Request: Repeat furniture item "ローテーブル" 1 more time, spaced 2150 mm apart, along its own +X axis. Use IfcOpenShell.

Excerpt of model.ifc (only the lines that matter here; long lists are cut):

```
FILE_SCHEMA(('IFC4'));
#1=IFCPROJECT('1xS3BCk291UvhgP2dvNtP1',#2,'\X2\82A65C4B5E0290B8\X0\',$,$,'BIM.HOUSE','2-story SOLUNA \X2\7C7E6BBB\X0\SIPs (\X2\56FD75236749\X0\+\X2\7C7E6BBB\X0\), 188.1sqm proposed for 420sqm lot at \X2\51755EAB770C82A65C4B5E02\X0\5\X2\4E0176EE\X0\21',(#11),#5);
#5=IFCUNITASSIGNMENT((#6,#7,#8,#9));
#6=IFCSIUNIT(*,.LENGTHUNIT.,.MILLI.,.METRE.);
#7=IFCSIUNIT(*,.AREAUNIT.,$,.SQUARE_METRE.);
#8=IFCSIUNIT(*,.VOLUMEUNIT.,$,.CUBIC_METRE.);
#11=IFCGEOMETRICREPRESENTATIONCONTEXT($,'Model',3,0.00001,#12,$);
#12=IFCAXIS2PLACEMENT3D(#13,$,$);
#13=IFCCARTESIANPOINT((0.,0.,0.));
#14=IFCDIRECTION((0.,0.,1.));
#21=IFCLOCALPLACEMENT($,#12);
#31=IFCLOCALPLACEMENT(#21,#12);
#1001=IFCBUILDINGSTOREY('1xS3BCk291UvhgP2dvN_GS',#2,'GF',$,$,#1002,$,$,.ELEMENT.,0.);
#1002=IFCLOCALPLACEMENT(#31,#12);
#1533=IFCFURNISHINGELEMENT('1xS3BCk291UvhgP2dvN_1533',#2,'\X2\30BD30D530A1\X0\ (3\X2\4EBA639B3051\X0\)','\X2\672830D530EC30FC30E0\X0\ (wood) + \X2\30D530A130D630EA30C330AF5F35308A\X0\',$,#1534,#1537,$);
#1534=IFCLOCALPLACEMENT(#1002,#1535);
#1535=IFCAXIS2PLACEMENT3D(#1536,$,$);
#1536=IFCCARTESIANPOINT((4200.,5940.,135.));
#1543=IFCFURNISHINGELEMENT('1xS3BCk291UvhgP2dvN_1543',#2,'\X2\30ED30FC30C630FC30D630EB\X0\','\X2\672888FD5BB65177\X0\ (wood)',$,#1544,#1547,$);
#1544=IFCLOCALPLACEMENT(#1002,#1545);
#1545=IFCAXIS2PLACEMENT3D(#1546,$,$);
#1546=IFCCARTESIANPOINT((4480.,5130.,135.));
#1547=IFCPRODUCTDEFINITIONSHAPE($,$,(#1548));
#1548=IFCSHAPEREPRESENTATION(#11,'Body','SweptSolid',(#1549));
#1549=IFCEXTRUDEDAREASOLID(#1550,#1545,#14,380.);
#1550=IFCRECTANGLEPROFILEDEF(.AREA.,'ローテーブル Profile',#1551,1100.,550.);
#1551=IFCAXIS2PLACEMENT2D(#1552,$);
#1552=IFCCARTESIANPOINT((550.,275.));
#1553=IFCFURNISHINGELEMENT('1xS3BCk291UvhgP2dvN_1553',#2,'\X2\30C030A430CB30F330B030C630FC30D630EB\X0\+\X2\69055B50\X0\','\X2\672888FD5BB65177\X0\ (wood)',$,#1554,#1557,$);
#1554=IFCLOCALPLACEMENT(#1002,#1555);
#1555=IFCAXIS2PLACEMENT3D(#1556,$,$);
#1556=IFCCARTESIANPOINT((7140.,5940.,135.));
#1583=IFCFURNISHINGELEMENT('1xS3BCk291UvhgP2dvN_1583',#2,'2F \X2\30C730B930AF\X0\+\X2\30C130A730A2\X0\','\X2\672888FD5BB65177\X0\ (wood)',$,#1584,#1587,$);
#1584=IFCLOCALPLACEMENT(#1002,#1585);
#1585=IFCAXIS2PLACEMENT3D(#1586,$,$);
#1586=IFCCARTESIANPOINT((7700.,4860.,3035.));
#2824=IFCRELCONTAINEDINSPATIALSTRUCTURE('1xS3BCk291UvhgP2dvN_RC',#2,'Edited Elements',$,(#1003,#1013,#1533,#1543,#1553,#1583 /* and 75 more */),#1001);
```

```python
import ifcopenshell
import ifcopenshell.api.geometry
import ifcopenshell.api.root
import ifcopenshell.util.element
import ifcopenshell.util.placement
import ifcopenshell.util.unit

model = ifcopenshell.open("model.ifc")
unit_scale = ifcopenshell.util.unit.calculate_unit_scale(model)


def reuse_history(source, copy):
    """copy_class also copies each property set's owner history, people and application; keep the originals."""
    for rel in copy.IsDefinedBy:
        if rel.is_a("IfcRelDefinesByProperties") and (history := rel.RelatingPropertyDefinition.OwnerHistory):
            rel.RelatingPropertyDefinition.OwnerHistory = source.OwnerHistory
            ifcopenshell.util.element.remove_deep2(model, history)


source = model.by_id(1543)
base = ifcopenshell.util.placement.get_local_placement(source.ObjectPlacement)
step = base[:3, 0] * 2.15 / unit_scale

for i in range(1, 2):
    copy = ifcopenshell.api.root.copy_class(model, product=source)
    copy.Representation = ifcopenshell.util.element.copy_deep(
        model, source.Representation, exclude=["IfcGeometricRepresentationContext", "IfcRepresentationMap"]
    )
    reuse_history(source, copy)
    matrix = base.copy()
    matrix[:3, 3] += i * step
    print("added at", matrix[:3, 3].round(3) + 0.0)
    ifcopenshell.api.geometry.edit_object_placement(model, product=copy, matrix=matrix, is_si=False)

model.write("model_rev.ifc")
```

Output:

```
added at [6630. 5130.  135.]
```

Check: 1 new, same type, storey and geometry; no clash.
